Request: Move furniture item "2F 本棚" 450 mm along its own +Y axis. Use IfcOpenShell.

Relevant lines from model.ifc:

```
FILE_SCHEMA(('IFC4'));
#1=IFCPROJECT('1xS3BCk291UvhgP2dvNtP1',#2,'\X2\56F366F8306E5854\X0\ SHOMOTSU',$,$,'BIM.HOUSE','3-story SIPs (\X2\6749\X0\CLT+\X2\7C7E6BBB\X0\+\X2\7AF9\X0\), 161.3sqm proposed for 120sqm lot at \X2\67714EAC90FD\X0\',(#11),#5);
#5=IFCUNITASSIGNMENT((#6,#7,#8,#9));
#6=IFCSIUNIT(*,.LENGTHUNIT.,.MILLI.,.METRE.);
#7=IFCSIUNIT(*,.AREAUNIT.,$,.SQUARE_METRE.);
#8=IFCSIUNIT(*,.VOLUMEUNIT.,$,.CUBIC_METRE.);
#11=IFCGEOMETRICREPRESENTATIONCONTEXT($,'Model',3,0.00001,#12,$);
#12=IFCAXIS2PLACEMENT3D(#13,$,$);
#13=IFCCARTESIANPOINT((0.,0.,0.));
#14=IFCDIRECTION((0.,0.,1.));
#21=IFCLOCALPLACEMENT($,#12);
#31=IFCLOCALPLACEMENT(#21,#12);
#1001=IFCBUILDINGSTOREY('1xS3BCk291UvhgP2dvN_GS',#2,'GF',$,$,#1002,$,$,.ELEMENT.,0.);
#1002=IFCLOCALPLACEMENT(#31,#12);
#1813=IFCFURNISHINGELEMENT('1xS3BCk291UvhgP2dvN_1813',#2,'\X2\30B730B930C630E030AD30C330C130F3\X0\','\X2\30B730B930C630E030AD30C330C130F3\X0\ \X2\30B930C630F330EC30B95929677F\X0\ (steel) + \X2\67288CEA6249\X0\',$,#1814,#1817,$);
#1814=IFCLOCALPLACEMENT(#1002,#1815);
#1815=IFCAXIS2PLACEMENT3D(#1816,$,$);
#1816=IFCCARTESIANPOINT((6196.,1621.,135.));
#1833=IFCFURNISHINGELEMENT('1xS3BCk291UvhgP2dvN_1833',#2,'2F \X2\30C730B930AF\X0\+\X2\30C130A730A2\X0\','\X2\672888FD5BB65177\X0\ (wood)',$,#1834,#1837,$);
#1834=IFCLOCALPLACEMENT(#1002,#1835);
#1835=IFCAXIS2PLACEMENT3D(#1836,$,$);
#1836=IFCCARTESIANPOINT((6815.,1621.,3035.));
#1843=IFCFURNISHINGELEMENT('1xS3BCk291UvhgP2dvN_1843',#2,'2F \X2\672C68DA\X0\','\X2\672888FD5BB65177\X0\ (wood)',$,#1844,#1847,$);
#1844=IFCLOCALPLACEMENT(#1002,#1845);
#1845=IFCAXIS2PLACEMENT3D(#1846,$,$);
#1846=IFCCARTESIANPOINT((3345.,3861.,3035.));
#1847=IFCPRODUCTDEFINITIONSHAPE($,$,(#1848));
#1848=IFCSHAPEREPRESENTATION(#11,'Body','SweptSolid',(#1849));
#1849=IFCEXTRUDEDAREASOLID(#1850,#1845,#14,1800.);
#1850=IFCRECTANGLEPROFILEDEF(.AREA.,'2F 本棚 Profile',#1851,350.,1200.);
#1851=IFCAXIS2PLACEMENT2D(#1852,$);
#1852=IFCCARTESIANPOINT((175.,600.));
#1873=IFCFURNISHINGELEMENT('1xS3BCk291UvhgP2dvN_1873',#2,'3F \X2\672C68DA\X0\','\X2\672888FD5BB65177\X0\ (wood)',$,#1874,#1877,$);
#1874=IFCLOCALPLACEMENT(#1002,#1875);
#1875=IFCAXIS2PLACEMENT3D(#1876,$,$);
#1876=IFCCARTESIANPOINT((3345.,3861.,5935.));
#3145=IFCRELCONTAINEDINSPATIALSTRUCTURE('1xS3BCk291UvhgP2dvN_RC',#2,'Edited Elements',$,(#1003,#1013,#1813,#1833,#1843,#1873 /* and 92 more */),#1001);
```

```python
import ifcopenshell
import ifcopenshell.api.geometry
import ifcopenshell.util.placement

model = ifcopenshell.open("model.ifc")

item = model.by_guid("1xS3BCk291UvhgP2dvN_1843")
matrix = ifcopenshell.util.placement.get_local_placement(item.ObjectPlacement)
matrix[:3, 3] += matrix[:3, 1] * 450.0
ifcopenshell.api.geometry.edit_object_placement(model, product=item, matrix=matrix, is_si=False)

print(ifcopenshell.util.placement.get_local_placement(item.ObjectPlacement).round(3) + 0.0)

model.write("model_rev.ifc")
```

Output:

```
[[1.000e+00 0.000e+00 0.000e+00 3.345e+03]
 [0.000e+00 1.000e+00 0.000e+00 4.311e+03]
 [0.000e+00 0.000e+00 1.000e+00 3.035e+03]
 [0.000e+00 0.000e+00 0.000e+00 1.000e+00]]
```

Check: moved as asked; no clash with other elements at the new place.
